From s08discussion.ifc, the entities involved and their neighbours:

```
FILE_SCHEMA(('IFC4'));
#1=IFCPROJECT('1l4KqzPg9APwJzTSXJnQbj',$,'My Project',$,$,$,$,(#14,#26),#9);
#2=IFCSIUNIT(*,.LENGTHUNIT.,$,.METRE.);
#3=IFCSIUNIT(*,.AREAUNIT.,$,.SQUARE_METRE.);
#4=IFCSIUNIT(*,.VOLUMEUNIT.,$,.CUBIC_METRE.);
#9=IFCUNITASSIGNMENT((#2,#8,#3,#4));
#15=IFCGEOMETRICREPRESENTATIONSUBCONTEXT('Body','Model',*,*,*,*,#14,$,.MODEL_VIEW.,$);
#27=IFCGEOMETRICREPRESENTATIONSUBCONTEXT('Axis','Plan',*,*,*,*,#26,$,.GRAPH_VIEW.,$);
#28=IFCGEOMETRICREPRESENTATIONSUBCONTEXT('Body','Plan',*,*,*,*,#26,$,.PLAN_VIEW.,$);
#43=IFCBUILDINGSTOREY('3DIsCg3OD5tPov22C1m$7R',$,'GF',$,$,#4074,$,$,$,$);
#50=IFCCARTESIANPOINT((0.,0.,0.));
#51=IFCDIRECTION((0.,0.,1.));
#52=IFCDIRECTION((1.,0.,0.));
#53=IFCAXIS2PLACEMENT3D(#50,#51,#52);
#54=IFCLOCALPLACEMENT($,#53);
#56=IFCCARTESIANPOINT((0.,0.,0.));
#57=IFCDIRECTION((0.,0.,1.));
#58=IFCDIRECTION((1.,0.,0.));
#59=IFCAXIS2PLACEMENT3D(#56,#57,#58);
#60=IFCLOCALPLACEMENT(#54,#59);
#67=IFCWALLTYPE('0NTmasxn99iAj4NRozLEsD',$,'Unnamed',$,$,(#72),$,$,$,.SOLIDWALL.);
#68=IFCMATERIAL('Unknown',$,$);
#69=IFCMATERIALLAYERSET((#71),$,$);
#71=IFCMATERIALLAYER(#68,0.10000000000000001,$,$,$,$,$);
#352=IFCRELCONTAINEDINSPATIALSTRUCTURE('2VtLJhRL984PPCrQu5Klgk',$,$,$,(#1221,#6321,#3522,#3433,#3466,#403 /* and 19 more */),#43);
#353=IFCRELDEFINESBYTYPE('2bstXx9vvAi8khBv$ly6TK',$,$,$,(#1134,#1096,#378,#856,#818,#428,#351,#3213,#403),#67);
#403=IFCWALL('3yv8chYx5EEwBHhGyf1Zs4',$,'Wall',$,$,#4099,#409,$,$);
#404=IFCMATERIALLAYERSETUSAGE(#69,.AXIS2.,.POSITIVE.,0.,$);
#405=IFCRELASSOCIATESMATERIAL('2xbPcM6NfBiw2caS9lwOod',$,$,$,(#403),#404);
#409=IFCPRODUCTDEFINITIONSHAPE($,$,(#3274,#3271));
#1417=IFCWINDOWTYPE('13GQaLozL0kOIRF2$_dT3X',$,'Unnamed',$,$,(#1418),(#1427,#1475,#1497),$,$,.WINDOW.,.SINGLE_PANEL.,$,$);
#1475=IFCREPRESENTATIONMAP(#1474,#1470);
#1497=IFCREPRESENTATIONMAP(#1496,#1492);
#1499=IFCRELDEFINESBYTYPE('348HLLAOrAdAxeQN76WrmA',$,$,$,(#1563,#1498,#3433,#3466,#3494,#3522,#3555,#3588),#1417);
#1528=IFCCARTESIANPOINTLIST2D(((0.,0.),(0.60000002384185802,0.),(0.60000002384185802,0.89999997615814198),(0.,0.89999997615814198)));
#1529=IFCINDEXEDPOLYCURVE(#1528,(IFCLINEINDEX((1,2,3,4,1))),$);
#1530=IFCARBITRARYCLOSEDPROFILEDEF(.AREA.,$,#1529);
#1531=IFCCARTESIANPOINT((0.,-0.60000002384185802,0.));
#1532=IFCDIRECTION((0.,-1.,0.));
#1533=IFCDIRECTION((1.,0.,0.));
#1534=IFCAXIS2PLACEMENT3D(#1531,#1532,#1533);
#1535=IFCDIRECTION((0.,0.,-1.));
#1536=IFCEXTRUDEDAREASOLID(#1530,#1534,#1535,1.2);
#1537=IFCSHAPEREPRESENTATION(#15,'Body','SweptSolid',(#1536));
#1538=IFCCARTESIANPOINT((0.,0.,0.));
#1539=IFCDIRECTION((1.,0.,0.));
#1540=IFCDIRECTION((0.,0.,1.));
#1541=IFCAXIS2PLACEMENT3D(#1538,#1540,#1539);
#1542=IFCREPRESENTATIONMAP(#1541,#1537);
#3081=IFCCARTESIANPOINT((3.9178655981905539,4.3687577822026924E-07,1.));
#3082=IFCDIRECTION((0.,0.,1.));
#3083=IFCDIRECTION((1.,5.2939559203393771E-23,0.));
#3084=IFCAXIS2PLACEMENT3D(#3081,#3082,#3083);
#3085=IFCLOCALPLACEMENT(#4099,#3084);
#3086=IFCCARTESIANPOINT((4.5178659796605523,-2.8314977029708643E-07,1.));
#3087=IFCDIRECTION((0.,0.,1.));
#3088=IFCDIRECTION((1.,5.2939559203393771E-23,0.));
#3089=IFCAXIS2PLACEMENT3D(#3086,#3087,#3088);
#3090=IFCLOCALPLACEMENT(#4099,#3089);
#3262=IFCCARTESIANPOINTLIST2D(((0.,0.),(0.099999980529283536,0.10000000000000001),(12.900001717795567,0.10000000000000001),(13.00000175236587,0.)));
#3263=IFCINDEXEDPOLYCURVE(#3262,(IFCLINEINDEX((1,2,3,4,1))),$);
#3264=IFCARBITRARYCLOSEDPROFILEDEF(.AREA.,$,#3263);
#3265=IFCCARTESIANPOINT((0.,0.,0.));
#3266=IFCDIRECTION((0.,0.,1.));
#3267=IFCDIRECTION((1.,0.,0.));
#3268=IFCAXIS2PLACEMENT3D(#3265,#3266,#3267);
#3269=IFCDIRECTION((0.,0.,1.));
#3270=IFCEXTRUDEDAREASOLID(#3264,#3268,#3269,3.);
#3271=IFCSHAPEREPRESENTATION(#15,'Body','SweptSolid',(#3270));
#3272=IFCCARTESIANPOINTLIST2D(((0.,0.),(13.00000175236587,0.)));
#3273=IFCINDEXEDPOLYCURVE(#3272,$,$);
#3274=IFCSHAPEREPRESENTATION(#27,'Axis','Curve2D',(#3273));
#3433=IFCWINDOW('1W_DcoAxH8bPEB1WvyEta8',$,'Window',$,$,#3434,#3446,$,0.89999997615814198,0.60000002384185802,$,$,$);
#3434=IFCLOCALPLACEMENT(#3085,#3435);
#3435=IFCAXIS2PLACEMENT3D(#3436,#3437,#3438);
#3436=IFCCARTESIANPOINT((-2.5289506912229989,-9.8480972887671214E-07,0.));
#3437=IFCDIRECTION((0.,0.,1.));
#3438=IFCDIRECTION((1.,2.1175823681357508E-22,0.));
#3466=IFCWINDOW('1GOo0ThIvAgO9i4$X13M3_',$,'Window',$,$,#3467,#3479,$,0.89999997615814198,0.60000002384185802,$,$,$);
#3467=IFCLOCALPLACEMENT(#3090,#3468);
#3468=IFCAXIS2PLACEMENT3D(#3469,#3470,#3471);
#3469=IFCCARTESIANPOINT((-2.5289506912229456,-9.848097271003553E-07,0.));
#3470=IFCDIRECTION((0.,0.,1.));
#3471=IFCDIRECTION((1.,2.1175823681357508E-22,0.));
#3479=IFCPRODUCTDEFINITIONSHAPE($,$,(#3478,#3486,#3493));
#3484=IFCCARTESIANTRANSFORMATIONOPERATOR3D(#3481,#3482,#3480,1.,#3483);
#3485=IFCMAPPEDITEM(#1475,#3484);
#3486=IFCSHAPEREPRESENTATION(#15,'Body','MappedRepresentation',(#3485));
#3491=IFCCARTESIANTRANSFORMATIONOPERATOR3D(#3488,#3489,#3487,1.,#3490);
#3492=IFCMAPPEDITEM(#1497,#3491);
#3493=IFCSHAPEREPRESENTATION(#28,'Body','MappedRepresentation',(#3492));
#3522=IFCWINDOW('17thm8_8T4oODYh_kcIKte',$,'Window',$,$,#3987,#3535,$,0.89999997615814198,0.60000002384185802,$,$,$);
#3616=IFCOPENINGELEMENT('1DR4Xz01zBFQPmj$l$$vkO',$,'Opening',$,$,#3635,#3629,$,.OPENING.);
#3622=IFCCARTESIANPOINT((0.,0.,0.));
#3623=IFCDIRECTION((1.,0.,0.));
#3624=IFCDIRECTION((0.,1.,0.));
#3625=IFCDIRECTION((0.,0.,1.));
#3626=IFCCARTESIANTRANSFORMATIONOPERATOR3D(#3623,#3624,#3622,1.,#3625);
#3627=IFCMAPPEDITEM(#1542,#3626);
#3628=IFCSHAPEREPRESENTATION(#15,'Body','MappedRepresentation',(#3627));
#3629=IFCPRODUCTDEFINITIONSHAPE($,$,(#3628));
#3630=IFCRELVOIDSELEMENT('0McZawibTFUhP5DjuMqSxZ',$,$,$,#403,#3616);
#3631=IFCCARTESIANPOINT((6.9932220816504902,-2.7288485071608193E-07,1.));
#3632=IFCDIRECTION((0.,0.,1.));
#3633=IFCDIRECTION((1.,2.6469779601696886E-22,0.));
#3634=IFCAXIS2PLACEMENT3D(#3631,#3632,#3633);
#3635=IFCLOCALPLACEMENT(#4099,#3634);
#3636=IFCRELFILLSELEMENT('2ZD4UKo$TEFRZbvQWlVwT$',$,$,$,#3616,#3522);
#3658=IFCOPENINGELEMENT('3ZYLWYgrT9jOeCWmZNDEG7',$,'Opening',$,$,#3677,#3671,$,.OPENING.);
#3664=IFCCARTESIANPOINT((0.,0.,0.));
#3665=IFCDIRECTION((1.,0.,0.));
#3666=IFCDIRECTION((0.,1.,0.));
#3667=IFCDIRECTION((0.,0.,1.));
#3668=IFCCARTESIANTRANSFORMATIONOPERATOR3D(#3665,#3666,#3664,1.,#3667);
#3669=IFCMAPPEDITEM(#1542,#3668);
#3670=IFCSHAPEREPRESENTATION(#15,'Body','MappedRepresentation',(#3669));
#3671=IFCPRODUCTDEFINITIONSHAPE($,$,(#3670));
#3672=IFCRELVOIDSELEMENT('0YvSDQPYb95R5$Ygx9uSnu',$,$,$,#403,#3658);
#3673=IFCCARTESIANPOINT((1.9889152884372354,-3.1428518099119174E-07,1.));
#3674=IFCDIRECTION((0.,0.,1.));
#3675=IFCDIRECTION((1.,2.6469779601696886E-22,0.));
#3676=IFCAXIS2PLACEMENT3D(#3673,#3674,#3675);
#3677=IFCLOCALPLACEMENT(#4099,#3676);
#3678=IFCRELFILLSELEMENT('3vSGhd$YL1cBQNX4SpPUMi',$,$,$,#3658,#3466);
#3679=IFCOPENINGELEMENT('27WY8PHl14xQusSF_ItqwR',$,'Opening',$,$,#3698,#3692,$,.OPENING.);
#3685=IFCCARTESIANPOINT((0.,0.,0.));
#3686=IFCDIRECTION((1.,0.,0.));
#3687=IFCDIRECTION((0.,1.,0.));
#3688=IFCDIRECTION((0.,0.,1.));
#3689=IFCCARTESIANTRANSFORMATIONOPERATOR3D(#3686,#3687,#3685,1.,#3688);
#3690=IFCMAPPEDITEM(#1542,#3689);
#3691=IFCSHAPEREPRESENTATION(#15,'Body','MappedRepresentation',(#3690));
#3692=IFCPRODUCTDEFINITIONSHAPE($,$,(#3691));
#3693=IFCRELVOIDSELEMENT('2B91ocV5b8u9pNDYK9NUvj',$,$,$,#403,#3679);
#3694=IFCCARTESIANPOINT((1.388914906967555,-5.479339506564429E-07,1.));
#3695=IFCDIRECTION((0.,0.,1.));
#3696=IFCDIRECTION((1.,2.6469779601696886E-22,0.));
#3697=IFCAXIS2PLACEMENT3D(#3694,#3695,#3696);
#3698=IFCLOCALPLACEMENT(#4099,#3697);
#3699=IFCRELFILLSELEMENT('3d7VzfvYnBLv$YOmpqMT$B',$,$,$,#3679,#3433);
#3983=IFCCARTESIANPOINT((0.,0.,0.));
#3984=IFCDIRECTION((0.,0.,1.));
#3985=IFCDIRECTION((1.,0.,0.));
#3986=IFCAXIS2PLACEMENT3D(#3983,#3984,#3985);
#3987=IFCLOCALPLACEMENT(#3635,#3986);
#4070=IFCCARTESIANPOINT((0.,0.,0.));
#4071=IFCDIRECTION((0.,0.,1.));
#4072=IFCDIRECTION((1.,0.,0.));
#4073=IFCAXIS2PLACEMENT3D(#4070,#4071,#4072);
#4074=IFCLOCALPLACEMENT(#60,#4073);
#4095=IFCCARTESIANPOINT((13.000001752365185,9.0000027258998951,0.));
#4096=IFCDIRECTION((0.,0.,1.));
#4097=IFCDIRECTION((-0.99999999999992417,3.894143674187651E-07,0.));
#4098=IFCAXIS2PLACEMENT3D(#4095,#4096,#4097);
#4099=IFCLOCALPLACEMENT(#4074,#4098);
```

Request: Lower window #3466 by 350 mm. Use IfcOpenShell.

```python
import numpy as np
import ifcopenshell
import ifcopenshell.api.geometry
import ifcopenshell.util.placement
import ifcopenshell.util.unit

model = ifcopenshell.open("s08discussion.ifc")
unit_scale = ifcopenshell.util.unit.calculate_unit_scale(model)

window = model.by_guid("1GOo0ThIvAgO9i4$X13M3_")
opening = window.FillsVoids[0].RelatingOpeningElement
dz = -0.35

shift = np.array([0.0, 0.0, dz])
# The window is not placed relative to its opening, so move both.
for product in (opening, window):
    matrix = ifcopenshell.util.placement.get_local_placement(product.ObjectPlacement)
    matrix[:3, 3] += shift
    ifcopenshell.api.geometry.edit_object_placement(model, product=product, matrix=matrix, is_si=False)

print(f"moved by {dz * unit_scale:+.3f} m")

model.write("s08discussion_rev.ifc")
```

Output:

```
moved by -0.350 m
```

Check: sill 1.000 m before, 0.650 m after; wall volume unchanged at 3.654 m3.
